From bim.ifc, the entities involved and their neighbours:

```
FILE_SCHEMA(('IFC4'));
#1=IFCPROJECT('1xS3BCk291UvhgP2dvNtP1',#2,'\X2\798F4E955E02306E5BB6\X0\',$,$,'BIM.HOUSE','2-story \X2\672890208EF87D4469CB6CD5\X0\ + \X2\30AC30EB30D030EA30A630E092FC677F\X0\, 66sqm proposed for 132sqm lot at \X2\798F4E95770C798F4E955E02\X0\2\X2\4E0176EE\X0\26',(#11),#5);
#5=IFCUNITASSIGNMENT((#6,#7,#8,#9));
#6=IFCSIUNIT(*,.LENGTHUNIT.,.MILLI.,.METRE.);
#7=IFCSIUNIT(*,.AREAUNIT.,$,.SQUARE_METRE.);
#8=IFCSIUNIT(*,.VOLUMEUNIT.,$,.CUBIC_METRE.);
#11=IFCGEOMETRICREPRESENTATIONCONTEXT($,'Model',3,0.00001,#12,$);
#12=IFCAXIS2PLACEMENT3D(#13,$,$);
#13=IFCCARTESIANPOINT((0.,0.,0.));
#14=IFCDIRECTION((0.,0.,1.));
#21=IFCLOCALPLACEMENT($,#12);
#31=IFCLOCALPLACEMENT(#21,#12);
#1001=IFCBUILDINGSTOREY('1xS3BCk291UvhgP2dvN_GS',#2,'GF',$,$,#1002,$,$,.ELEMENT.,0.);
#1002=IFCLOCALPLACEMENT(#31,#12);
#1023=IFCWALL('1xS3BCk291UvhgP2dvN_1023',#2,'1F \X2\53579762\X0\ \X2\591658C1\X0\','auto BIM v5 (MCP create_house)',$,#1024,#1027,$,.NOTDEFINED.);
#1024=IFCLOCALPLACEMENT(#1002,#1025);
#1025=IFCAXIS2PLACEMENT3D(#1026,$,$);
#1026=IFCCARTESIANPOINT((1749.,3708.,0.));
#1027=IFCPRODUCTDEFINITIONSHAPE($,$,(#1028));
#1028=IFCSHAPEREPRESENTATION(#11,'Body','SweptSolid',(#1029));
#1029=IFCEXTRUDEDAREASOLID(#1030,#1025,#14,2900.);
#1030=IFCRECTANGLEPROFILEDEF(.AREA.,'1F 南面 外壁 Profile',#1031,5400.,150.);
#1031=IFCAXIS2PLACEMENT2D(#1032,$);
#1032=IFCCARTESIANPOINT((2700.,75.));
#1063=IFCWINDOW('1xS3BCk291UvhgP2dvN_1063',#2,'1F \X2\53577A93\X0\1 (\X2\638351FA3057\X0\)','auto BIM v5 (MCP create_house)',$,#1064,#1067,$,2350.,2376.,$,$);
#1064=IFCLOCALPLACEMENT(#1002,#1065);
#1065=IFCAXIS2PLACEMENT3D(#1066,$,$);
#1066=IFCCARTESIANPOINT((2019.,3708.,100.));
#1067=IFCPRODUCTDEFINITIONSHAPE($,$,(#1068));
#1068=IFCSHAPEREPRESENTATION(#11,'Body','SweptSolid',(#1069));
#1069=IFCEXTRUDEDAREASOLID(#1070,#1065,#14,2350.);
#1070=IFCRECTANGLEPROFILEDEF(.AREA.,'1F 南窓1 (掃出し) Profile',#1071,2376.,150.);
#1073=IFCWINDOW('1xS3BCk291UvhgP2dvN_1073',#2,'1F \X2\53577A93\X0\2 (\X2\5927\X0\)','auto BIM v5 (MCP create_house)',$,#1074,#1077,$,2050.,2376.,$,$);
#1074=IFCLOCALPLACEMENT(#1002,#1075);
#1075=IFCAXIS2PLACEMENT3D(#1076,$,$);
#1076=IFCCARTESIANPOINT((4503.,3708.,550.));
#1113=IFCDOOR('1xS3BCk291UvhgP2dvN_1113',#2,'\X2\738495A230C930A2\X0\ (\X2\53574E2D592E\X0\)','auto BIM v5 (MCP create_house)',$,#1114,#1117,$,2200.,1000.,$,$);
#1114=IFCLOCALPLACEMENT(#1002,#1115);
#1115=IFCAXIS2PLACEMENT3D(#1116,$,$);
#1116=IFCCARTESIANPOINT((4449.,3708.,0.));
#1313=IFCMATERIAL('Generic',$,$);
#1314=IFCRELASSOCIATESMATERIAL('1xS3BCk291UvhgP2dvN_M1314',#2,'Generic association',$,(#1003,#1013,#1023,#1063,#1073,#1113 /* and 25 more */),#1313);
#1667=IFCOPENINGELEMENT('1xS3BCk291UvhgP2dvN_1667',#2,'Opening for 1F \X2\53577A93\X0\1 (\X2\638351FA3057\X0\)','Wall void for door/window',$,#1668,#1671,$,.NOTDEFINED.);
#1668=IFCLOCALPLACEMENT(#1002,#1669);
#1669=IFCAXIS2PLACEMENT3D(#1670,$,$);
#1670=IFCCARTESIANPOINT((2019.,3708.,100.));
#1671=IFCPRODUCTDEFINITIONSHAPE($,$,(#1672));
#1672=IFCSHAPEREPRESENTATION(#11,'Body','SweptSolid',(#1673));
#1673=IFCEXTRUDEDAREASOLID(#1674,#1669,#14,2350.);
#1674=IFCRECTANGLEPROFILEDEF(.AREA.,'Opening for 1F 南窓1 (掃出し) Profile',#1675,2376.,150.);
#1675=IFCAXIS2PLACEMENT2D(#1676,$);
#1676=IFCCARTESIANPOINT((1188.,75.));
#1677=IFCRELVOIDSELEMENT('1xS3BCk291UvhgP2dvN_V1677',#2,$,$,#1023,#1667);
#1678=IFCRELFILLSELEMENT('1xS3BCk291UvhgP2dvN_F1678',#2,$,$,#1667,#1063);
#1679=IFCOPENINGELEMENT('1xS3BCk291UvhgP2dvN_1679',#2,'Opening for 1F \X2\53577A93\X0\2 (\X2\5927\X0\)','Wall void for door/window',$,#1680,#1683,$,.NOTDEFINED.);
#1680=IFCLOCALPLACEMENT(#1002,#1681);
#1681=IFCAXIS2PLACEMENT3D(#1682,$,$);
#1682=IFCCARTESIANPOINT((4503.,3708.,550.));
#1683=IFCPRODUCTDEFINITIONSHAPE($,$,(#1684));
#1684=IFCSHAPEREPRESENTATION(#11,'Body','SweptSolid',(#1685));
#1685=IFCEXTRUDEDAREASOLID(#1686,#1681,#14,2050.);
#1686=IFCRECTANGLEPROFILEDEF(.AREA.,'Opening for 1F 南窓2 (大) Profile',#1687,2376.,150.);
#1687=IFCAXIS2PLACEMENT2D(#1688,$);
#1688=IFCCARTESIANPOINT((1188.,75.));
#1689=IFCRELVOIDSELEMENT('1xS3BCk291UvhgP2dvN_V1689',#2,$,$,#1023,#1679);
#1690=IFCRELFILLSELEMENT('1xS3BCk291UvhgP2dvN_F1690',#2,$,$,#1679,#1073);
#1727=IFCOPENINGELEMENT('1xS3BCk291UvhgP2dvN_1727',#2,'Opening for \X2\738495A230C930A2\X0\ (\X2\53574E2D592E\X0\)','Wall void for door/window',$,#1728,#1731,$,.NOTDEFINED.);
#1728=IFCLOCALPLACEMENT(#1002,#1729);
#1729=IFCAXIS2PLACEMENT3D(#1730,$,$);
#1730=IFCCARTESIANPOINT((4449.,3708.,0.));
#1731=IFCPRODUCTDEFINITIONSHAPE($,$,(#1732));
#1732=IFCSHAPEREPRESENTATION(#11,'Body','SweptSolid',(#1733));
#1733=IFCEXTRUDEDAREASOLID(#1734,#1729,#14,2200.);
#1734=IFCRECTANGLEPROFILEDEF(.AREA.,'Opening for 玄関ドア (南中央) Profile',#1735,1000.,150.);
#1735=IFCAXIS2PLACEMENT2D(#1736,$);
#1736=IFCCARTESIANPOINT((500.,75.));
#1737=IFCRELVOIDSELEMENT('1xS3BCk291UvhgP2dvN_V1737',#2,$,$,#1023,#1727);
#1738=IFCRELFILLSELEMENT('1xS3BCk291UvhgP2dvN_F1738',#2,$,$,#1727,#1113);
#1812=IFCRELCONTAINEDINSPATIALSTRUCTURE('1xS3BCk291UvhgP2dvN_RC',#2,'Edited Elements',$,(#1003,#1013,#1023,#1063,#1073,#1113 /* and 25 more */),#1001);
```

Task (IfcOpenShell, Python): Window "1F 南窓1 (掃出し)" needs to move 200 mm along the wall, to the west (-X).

```python
import ifcopenshell
import ifcopenshell.api.geometry
import ifcopenshell.util.placement

model = ifcopenshell.open("bim.ifc")

window = model.by_guid("1xS3BCk291UvhgP2dvN_1063")
opening = window.FillsVoids[0].RelatingOpeningElement
wall = opening.VoidsElements[0].RelatingBuildingElement

wall_matrix = ifcopenshell.util.placement.get_local_placement(wall.ObjectPlacement)
shift = wall_matrix[:3, 0] * -200.0
before = ifcopenshell.util.placement.get_local_placement(window.ObjectPlacement)[:3, 3].copy()

# The window is not placed relative to its opening, so move both.
for product in (opening, window):
    matrix = ifcopenshell.util.placement.get_local_placement(product.ObjectPlacement)
    matrix[:3, 3] += shift
    ifcopenshell.api.geometry.edit_object_placement(model, product=product, matrix=matrix, is_si=False)

after = ifcopenshell.util.placement.get_local_placement(window.ObjectPlacement)[:3, 3]
print("window moved by", (after - before).round(3) + 0.0)

model.write("bim_updated.ifc")
```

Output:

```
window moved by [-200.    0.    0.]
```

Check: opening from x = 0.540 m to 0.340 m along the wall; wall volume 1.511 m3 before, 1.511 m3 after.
